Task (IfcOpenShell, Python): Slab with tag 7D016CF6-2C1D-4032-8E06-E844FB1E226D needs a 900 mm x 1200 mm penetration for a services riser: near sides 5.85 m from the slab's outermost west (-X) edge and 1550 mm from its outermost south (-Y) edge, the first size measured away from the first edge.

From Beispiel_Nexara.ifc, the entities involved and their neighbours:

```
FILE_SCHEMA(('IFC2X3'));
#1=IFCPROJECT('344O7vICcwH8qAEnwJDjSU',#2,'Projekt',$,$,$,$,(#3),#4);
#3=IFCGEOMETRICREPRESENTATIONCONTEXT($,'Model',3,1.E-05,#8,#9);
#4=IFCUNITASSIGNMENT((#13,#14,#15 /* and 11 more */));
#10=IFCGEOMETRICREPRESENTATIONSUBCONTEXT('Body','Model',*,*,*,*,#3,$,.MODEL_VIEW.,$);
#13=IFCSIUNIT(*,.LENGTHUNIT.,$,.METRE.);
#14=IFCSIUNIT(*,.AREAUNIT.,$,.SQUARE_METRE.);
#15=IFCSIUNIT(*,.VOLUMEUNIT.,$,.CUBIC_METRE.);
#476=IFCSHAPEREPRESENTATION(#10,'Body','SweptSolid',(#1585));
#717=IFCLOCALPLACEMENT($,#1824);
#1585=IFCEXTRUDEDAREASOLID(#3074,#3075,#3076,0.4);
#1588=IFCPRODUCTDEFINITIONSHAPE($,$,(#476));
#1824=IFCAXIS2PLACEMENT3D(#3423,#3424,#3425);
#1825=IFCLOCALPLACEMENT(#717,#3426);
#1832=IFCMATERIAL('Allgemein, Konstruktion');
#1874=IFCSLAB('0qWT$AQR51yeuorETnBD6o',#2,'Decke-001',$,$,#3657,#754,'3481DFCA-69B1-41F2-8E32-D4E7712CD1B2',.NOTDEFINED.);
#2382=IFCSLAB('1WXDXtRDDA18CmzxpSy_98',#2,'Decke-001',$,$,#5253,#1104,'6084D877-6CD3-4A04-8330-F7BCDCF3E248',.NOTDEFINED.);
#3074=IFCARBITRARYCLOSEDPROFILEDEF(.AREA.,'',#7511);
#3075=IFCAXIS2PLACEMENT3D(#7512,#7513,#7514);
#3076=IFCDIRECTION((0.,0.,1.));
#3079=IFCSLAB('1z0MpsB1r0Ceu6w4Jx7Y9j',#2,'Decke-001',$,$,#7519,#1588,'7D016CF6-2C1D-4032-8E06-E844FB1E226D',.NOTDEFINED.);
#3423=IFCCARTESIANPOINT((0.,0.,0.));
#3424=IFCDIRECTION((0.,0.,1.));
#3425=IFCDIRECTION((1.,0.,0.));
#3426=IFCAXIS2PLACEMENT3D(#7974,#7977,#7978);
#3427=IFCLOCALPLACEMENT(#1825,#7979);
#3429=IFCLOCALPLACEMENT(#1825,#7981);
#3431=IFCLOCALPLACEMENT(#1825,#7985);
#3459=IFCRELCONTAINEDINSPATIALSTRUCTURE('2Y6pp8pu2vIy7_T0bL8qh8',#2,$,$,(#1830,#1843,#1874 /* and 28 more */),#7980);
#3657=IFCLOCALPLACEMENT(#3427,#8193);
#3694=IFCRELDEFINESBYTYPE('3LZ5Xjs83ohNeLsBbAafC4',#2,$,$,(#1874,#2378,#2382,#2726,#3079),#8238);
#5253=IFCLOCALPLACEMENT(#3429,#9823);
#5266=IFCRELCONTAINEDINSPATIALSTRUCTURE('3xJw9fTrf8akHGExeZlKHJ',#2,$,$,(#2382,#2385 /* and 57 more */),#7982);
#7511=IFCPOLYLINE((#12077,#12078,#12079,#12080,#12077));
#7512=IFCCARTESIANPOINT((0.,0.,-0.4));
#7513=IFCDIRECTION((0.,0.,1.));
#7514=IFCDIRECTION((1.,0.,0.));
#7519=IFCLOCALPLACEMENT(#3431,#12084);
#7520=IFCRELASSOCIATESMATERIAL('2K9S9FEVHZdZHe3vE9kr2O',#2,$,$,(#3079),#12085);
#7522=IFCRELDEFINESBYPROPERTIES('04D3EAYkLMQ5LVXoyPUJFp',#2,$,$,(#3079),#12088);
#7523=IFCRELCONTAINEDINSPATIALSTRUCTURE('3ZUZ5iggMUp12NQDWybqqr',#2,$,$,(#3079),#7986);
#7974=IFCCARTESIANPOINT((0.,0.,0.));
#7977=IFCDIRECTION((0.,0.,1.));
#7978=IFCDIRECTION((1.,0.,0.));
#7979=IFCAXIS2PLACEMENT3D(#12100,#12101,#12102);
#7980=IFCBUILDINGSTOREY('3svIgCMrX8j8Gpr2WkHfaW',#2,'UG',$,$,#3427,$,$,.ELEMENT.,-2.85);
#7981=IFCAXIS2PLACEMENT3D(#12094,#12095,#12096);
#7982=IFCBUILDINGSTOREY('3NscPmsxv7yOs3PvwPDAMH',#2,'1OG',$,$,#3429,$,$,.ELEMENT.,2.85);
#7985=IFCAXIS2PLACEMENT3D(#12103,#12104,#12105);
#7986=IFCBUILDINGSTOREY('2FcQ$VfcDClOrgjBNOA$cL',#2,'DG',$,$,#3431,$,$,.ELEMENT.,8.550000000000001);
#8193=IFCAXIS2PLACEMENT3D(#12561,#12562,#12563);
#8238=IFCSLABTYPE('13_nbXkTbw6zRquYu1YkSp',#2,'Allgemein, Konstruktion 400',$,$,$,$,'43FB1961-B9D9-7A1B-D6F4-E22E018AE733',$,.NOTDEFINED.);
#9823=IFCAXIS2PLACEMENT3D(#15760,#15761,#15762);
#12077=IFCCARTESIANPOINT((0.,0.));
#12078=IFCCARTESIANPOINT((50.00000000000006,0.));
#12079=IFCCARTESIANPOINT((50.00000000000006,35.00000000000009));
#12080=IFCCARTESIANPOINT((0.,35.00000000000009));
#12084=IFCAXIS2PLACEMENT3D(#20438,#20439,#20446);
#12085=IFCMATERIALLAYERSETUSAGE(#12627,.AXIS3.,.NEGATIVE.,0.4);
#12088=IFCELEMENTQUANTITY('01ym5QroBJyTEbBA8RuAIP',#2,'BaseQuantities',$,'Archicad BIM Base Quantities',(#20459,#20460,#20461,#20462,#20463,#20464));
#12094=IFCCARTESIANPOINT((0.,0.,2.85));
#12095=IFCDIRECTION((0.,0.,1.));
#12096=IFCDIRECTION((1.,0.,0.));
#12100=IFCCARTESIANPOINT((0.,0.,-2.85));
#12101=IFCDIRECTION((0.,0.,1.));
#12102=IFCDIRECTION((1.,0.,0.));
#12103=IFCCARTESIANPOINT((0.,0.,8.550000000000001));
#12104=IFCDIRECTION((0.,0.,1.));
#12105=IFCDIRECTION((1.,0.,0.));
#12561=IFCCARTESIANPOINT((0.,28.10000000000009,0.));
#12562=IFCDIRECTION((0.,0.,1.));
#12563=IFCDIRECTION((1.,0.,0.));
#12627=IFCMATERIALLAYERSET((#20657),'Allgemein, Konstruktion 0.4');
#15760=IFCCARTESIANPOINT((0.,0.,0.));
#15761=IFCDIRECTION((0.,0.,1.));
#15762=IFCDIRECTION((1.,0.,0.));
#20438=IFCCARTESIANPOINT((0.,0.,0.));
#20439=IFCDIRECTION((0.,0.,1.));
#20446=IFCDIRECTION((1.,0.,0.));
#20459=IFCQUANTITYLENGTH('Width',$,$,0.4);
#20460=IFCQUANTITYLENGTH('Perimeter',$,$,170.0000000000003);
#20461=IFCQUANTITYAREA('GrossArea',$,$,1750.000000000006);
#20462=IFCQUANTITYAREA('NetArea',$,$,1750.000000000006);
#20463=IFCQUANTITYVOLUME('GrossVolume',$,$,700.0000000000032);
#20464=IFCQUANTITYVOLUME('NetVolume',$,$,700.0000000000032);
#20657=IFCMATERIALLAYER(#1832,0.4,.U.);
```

```python
import numpy as np
import ifcopenshell
import ifcopenshell.api.feature
import ifcopenshell.api.geometry
import ifcopenshell.api.pset
import ifcopenshell.api.root
import ifcopenshell.geom
import ifcopenshell.util.element
import ifcopenshell.util.placement
import ifcopenshell.util.representation
import ifcopenshell.util.shape
import ifcopenshell.util.unit

model = ifcopenshell.open("Beispiel_Nexara.ifc")
unit_scale = ifcopenshell.util.unit.calculate_unit_scale(model)
area_scale = ifcopenshell.util.unit.calculate_unit_scale(model, "AREAUNIT")
volume_scale = ifcopenshell.util.unit.calculate_unit_scale(model, "VOLUMEUNIT")
settings = ifcopenshell.geom.settings()


def volume(element):
    """Net volume in cubic metres, openings subtracted."""
    shape = ifcopenshell.geom.create_shape(settings, element)
    return ifcopenshell.util.shape.get_volume(shape.geometry)


slab = model.by_id(3079)
before = volume(slab)

# Extent in the slab's own axes, in metres. The edges named are its -X and -Y sides.
slab_shape = ifcopenshell.geom.create_shape(settings, slab)
vertices = ifcopenshell.util.shape.get_vertices(slab_shape.geometry)
x_min, y_min, bottom = vertices.min(axis=0)
top = vertices[:, 2].max()

opening = ifcopenshell.api.root.create_entity(model, ifc_class="IfcOpeningElement", name="Services riser opening")
context = ifcopenshell.util.representation.get_context(model, "Model", "Body", "MODEL_VIEW")
width, depth = 0.9, 1.2
outline = [(0.0, 0.0), (width, 0.0), (width, depth), (0.0, depth), (0.0, 0.0)]
# Overshoot both faces by 50 mm so the cut is clean.
shape = ifcopenshell.api.geometry.add_slab_representation(
    model, context=context, depth=top - bottom + 0.1, polyline=outline
)
ifcopenshell.api.geometry.assign_representation(model, product=opening, representation=shape)

matrix = ifcopenshell.util.placement.get_local_placement(slab.ObjectPlacement)
matrix[:, 3] = matrix @ np.append(np.array([x_min + 5.85, y_min + 1.55, bottom - 0.05]) / unit_scale, 1.0)
ifcopenshell.api.geometry.edit_object_placement(model, product=opening, matrix=matrix, is_si=False)
ifcopenshell.api.feature.add_feature(model, feature=opening, element=slab)

after = volume(slab)

# Update the slab's stored quantities.
qto = model.by_id(ifcopenshell.util.element.get_pset(slab, "BaseQuantities", should_inherit=False)["id"])
ifcopenshell.api.pset.edit_qto(model, qto=qto, properties={
    "NetArea": after / (top - bottom) / area_scale,
    "NetVolume": after / volume_scale,
})

print(f"slab volume {before:.3f} -> {after:.3f} m3")

model.write("Beispiel_Nexara_v2.ifc")
```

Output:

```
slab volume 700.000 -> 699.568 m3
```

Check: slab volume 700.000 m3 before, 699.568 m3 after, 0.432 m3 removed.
